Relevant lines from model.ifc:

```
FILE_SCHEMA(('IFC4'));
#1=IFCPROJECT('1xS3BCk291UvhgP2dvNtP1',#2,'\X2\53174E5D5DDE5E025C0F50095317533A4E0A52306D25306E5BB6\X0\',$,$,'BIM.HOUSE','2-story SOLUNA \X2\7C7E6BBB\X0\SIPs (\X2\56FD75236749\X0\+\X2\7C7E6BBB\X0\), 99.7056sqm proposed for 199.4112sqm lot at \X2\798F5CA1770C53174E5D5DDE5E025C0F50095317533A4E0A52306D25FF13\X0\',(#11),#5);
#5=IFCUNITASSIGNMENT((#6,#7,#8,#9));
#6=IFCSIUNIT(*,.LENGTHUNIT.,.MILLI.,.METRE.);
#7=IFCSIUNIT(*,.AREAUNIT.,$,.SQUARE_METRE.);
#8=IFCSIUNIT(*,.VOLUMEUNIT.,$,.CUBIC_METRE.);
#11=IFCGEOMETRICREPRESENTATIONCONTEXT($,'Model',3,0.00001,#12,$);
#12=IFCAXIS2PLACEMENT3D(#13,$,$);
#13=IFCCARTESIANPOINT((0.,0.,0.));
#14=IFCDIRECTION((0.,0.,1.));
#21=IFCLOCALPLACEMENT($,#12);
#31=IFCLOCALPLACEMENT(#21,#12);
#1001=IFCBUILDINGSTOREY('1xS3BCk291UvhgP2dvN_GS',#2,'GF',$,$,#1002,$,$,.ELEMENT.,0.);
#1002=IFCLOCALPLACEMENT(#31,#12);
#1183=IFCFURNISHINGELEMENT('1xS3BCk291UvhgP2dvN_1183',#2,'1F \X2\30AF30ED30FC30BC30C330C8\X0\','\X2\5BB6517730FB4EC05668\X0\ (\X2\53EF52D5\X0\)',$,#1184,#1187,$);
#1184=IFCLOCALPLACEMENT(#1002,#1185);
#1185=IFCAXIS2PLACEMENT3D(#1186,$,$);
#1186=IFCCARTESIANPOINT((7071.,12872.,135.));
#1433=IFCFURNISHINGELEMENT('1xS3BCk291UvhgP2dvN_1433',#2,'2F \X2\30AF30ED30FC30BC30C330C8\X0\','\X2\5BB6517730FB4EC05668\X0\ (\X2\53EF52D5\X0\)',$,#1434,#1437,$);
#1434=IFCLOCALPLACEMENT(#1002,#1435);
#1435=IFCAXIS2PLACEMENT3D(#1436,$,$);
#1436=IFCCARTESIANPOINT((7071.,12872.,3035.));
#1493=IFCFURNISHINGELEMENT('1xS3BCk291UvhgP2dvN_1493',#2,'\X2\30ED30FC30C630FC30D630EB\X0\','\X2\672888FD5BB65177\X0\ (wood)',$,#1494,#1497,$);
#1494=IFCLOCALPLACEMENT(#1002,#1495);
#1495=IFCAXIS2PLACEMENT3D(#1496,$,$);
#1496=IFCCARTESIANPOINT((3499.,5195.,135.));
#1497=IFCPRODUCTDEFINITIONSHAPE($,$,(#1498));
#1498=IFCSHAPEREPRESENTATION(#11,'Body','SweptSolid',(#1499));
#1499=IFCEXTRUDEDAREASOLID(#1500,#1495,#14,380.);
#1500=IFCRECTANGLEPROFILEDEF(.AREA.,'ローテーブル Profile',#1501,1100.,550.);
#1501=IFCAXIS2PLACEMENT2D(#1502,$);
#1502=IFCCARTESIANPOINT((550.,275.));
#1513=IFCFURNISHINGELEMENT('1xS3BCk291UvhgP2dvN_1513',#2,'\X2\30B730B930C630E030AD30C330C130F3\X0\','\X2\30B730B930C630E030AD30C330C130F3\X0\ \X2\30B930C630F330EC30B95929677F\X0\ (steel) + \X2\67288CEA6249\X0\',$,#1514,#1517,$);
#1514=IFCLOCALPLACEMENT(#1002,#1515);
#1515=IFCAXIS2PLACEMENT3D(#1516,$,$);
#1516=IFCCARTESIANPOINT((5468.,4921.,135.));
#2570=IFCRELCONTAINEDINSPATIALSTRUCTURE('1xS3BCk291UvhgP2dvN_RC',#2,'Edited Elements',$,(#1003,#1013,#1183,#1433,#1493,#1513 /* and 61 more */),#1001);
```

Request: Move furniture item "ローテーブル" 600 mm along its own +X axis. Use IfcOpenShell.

```python
import ifcopenshell
import ifcopenshell.api.geometry
import ifcopenshell.util.placement
import ifcopenshell.util.unit

model = ifcopenshell.open("model.ifc")
unit_scale = ifcopenshell.util.unit.calculate_unit_scale(model)

item = model.by_guid("1xS3BCk291UvhgP2dvN_1493")
matrix = ifcopenshell.util.placement.get_local_placement(item.ObjectPlacement)
matrix[:3, 3] += matrix[:3, 0] * 0.6 / unit_scale
ifcopenshell.api.geometry.edit_object_placement(model, product=item, matrix=matrix, is_si=False)

print(ifcopenshell.util.placement.get_local_placement(item.ObjectPlacement).round(3) + 0.0)

model.write("model_rev.ifc")
```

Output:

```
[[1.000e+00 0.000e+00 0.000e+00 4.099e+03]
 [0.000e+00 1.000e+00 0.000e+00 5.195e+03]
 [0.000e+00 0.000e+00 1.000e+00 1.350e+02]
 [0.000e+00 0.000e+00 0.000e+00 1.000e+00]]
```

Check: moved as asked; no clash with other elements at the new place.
